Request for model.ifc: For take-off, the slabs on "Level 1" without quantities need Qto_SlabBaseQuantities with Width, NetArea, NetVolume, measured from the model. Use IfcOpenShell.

First a look at what the model holds.

```python
import ifcopenshell
import ifcopenshell.util.element
import ifcopenshell.util.unit

model = ifcopenshell.open("model.ifc")
print(model.schema)
for unit_type in ("LENGTHUNIT", "AREAUNIT", "VOLUMEUNIT"):
    print(unit_type, ifcopenshell.util.unit.calculate_unit_scale(model, unit_type))
storey = next(s for s in model.by_type("IfcBuildingStorey") if s.Name == "Level 1")
slabs = [e for e in ifcopenshell.util.element.get_decomposition(storey) if e.is_a("IfcSlab")]
for e in sorted(slabs, key=lambda e: e.id()):
    print(e.id(), e.is_a(), e.Name, list(ifcopenshell.util.element.get_psets(e, qtos_only=True)), sep=" | ")
```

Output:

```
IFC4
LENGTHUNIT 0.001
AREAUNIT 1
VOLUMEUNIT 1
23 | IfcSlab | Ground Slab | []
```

```python
import ifcopenshell
import ifcopenshell.api.pset
import ifcopenshell.geom
import ifcopenshell.util.element
import ifcopenshell.util.shape
import ifcopenshell.util.unit

model = ifcopenshell.open("model.ifc")
unit_scale = ifcopenshell.util.unit.calculate_unit_scale(model)
area_scale = ifcopenshell.util.unit.calculate_unit_scale(model, "AREAUNIT")
volume_scale = ifcopenshell.util.unit.calculate_unit_scale(model, "VOLUMEUNIT")
settings = ifcopenshell.geom.settings()

storey = next(s for s in model.by_type("IfcBuildingStorey") if s.Name == "Level 1")
slabs = [e for e in ifcopenshell.util.element.get_decomposition(storey) if e.is_a("IfcSlab")]

for e in sorted(slabs, key=lambda e: e.id()):
    if ifcopenshell.util.element.get_psets(e, qtos_only=True, should_inherit=False):
        continue
    # Geometry comes back in metres, in the element's own axes.
    shape = ifcopenshell.geom.create_shape(settings, e)
    values = {
        "Width": ifcopenshell.util.shape.get_z(shape.geometry) / unit_scale,
        "NetArea": ifcopenshell.util.shape.get_footprint_area(shape.geometry) / area_scale,
        "NetVolume": ifcopenshell.util.shape.get_volume(shape.geometry) / volume_scale,
    }
    qto = ifcopenshell.api.pset.add_qto(model, product=e, name="Qto_SlabBaseQuantities")
    ifcopenshell.api.pset.edit_qto(model, qto=qto, properties=values)
    print(e.id(), {k: round(v, 3) for k, v in values.items()})

model.write("model-out.ifc")
```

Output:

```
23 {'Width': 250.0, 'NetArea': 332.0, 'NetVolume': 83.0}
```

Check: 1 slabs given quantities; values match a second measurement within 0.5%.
